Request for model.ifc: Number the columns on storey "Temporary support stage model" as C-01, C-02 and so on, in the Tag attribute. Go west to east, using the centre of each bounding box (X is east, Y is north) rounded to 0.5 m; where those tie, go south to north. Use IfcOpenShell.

First a look at what the model holds.

```python
import ifcopenshell
import ifcopenshell.util.element
import ifcopenshell.util.placement

model = ifcopenshell.open("model.ifc")
print(model.schema)
storey = next(s for s in model.by_type("IfcBuildingStorey") if s.Name == "Temporary support stage model")
columns = [e for e in ifcopenshell.util.element.get_decomposition(storey) if e.is_a("IfcColumn")]
for e in sorted(columns, key=lambda e: e.id()):
    origin = ifcopenshell.util.placement.get_local_placement(e.ObjectPlacement)[:3, 3]
    print(e.id(), e.Tag, e.Name, origin.round(2) + 0.0, sep=" | ")
```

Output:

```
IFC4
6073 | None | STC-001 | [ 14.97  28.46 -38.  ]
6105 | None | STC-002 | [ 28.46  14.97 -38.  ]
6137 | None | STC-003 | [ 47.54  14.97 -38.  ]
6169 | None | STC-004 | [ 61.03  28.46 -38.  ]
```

```python
import ifcopenshell
import ifcopenshell.geom
import ifcopenshell.util.element
import ifcopenshell.util.shape

model = ifcopenshell.open("model.ifc")
settings = ifcopenshell.geom.settings()
settings.set("use-world-coords", True)


def centre(element):
    shape = ifcopenshell.geom.create_shape(settings, element)
    return ifcopenshell.util.shape.get_bbox_centroid(shape.geometry)


storey = next(s for s in model.by_type("IfcBuildingStorey") if s.Name == "Temporary support stage model")
columns = [e for e in ifcopenshell.util.element.get_decomposition(storey) if e.is_a("IfcColumn")]

# Insertion points can sit at a corner or the storey origin, so sort by the geometry (in metres).
centres = {e: centre(e) for e in columns}
columns.sort(key=lambda e: (round(centres[e][0] / 0.5), centres[e][1]))

for i, e in enumerate(columns, start=1):
    number = f"C-{i:02d}"
    e.Tag = number
    print(e.id(), number)

model.write("model_rev.ifc")
```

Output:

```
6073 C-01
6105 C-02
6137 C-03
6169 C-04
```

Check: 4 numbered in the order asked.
